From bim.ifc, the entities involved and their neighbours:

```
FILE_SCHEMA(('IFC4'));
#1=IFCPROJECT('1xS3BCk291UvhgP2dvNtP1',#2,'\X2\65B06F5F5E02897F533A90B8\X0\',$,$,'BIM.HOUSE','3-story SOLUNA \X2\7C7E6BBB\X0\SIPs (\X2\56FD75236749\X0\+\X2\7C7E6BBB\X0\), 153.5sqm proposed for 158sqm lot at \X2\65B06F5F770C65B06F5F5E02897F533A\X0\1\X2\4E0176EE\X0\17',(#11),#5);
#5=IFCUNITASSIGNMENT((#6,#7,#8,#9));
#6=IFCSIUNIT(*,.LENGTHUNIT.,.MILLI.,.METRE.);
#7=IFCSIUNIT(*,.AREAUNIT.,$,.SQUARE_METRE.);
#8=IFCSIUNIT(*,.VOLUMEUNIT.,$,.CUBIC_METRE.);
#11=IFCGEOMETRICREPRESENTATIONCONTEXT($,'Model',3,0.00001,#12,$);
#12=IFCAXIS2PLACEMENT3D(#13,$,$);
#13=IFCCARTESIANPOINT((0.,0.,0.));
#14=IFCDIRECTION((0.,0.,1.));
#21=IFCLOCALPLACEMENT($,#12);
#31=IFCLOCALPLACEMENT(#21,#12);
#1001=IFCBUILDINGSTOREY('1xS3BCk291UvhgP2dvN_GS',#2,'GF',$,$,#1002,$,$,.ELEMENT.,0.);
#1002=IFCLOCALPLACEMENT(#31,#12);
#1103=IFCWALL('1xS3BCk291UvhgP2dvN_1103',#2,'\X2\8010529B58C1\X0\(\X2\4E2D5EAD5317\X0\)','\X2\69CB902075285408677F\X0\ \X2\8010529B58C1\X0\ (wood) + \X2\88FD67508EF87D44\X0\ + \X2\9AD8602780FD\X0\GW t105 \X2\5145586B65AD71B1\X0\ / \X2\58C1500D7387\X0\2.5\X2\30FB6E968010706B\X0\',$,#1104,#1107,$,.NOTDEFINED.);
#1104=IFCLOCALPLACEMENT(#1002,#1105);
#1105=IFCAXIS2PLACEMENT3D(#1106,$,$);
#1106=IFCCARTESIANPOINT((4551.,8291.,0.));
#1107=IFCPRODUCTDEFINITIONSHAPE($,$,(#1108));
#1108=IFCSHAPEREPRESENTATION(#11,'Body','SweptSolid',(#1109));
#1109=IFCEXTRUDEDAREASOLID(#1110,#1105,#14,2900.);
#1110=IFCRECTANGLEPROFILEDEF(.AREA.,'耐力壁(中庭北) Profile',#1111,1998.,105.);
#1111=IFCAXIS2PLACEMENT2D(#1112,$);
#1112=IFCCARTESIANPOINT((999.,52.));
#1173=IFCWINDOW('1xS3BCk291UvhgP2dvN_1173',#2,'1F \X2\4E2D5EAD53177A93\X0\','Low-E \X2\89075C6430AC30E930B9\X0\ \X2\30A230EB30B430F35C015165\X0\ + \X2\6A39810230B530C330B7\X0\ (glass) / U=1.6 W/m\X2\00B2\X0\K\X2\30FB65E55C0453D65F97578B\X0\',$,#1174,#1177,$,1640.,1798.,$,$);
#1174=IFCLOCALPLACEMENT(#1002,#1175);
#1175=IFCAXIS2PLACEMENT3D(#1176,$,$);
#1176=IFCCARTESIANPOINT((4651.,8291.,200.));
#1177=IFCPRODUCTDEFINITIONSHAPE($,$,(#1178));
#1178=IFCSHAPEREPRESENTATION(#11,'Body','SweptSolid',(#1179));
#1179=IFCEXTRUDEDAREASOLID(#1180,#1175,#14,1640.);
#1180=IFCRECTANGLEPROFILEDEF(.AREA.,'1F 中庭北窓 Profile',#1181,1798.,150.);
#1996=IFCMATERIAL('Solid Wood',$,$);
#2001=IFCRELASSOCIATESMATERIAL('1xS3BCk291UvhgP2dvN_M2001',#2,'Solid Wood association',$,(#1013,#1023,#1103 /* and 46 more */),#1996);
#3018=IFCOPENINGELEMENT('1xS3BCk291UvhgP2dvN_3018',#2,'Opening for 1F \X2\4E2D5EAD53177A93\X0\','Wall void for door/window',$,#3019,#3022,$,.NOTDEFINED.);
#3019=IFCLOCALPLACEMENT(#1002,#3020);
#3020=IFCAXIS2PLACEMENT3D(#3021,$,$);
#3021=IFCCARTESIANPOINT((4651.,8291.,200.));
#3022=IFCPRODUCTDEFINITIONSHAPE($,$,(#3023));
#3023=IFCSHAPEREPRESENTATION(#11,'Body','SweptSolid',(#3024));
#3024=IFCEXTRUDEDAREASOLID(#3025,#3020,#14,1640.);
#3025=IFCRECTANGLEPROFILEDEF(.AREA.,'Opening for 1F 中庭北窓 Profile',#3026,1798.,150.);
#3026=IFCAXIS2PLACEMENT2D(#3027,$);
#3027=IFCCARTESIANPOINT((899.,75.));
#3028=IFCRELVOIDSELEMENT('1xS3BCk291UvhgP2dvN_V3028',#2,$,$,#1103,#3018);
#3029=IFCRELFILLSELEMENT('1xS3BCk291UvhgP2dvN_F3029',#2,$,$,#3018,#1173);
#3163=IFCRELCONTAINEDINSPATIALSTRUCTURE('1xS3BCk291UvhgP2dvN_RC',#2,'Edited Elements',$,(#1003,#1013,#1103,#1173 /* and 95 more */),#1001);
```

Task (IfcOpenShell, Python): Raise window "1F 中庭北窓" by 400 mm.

```python
import numpy as np
import ifcopenshell
import ifcopenshell.api.geometry
import ifcopenshell.util.placement
import ifcopenshell.util.unit

model = ifcopenshell.open("bim.ifc")
unit_scale = ifcopenshell.util.unit.calculate_unit_scale(model)

window = model.by_guid("1xS3BCk291UvhgP2dvN_1173")
opening = window.FillsVoids[0].RelatingOpeningElement
dz = 0.4 / unit_scale

shift = np.array([0.0, 0.0, dz])
# The window is not placed relative to its opening, so move both.
for product in (opening, window):
    matrix = ifcopenshell.util.placement.get_local_placement(product.ObjectPlacement)
    matrix[:3, 3] += shift
    ifcopenshell.api.geometry.edit_object_placement(model, product=product, matrix=matrix, is_si=False)

print(f"moved by {dz * unit_scale:+.3f} m")

model.write("bim_edited.ifc")
```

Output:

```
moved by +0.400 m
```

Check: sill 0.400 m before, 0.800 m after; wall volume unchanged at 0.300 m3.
